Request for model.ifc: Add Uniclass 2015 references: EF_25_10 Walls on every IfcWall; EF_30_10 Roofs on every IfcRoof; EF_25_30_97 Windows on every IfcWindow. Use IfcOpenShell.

First a look at what the model holds.

```python
import ifcopenshell

model = ifcopenshell.open("model.ifc")
print(model.schema)
print("classifications:", [c.Name for c in model.by_type("IfcClassification")])
for ifc_class in ("IfcDoor", "IfcRoof", "IfcStair", "IfcWall", "IfcWindow"):
    print(ifc_class, len(model.by_type(ifc_class)))
```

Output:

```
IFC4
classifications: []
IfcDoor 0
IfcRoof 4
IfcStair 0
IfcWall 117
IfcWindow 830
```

```python
import ifcopenshell
import ifcopenshell.api.classification

model = ifcopenshell.open("model.ifc")

system = ifcopenshell.api.classification.add_classification(model, classification="Uniclass 2015")

codes = {
    "IfcWall": ("EF_25_10", "Walls"),
    "IfcRoof": ("EF_30_10", "Roofs"),
    "IfcWindow": ("EF_25_30_97", "Windows"),
}
for ifc_class, (code, name) in codes.items():
    products = model.by_type(ifc_class)
    ifcopenshell.api.classification.add_reference(
        model, products=products, classification=system, identification=code, name=name
    )
    print(code, len(products))

model.write("model_updated.ifc")
```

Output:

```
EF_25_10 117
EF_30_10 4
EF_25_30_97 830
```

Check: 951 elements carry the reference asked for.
